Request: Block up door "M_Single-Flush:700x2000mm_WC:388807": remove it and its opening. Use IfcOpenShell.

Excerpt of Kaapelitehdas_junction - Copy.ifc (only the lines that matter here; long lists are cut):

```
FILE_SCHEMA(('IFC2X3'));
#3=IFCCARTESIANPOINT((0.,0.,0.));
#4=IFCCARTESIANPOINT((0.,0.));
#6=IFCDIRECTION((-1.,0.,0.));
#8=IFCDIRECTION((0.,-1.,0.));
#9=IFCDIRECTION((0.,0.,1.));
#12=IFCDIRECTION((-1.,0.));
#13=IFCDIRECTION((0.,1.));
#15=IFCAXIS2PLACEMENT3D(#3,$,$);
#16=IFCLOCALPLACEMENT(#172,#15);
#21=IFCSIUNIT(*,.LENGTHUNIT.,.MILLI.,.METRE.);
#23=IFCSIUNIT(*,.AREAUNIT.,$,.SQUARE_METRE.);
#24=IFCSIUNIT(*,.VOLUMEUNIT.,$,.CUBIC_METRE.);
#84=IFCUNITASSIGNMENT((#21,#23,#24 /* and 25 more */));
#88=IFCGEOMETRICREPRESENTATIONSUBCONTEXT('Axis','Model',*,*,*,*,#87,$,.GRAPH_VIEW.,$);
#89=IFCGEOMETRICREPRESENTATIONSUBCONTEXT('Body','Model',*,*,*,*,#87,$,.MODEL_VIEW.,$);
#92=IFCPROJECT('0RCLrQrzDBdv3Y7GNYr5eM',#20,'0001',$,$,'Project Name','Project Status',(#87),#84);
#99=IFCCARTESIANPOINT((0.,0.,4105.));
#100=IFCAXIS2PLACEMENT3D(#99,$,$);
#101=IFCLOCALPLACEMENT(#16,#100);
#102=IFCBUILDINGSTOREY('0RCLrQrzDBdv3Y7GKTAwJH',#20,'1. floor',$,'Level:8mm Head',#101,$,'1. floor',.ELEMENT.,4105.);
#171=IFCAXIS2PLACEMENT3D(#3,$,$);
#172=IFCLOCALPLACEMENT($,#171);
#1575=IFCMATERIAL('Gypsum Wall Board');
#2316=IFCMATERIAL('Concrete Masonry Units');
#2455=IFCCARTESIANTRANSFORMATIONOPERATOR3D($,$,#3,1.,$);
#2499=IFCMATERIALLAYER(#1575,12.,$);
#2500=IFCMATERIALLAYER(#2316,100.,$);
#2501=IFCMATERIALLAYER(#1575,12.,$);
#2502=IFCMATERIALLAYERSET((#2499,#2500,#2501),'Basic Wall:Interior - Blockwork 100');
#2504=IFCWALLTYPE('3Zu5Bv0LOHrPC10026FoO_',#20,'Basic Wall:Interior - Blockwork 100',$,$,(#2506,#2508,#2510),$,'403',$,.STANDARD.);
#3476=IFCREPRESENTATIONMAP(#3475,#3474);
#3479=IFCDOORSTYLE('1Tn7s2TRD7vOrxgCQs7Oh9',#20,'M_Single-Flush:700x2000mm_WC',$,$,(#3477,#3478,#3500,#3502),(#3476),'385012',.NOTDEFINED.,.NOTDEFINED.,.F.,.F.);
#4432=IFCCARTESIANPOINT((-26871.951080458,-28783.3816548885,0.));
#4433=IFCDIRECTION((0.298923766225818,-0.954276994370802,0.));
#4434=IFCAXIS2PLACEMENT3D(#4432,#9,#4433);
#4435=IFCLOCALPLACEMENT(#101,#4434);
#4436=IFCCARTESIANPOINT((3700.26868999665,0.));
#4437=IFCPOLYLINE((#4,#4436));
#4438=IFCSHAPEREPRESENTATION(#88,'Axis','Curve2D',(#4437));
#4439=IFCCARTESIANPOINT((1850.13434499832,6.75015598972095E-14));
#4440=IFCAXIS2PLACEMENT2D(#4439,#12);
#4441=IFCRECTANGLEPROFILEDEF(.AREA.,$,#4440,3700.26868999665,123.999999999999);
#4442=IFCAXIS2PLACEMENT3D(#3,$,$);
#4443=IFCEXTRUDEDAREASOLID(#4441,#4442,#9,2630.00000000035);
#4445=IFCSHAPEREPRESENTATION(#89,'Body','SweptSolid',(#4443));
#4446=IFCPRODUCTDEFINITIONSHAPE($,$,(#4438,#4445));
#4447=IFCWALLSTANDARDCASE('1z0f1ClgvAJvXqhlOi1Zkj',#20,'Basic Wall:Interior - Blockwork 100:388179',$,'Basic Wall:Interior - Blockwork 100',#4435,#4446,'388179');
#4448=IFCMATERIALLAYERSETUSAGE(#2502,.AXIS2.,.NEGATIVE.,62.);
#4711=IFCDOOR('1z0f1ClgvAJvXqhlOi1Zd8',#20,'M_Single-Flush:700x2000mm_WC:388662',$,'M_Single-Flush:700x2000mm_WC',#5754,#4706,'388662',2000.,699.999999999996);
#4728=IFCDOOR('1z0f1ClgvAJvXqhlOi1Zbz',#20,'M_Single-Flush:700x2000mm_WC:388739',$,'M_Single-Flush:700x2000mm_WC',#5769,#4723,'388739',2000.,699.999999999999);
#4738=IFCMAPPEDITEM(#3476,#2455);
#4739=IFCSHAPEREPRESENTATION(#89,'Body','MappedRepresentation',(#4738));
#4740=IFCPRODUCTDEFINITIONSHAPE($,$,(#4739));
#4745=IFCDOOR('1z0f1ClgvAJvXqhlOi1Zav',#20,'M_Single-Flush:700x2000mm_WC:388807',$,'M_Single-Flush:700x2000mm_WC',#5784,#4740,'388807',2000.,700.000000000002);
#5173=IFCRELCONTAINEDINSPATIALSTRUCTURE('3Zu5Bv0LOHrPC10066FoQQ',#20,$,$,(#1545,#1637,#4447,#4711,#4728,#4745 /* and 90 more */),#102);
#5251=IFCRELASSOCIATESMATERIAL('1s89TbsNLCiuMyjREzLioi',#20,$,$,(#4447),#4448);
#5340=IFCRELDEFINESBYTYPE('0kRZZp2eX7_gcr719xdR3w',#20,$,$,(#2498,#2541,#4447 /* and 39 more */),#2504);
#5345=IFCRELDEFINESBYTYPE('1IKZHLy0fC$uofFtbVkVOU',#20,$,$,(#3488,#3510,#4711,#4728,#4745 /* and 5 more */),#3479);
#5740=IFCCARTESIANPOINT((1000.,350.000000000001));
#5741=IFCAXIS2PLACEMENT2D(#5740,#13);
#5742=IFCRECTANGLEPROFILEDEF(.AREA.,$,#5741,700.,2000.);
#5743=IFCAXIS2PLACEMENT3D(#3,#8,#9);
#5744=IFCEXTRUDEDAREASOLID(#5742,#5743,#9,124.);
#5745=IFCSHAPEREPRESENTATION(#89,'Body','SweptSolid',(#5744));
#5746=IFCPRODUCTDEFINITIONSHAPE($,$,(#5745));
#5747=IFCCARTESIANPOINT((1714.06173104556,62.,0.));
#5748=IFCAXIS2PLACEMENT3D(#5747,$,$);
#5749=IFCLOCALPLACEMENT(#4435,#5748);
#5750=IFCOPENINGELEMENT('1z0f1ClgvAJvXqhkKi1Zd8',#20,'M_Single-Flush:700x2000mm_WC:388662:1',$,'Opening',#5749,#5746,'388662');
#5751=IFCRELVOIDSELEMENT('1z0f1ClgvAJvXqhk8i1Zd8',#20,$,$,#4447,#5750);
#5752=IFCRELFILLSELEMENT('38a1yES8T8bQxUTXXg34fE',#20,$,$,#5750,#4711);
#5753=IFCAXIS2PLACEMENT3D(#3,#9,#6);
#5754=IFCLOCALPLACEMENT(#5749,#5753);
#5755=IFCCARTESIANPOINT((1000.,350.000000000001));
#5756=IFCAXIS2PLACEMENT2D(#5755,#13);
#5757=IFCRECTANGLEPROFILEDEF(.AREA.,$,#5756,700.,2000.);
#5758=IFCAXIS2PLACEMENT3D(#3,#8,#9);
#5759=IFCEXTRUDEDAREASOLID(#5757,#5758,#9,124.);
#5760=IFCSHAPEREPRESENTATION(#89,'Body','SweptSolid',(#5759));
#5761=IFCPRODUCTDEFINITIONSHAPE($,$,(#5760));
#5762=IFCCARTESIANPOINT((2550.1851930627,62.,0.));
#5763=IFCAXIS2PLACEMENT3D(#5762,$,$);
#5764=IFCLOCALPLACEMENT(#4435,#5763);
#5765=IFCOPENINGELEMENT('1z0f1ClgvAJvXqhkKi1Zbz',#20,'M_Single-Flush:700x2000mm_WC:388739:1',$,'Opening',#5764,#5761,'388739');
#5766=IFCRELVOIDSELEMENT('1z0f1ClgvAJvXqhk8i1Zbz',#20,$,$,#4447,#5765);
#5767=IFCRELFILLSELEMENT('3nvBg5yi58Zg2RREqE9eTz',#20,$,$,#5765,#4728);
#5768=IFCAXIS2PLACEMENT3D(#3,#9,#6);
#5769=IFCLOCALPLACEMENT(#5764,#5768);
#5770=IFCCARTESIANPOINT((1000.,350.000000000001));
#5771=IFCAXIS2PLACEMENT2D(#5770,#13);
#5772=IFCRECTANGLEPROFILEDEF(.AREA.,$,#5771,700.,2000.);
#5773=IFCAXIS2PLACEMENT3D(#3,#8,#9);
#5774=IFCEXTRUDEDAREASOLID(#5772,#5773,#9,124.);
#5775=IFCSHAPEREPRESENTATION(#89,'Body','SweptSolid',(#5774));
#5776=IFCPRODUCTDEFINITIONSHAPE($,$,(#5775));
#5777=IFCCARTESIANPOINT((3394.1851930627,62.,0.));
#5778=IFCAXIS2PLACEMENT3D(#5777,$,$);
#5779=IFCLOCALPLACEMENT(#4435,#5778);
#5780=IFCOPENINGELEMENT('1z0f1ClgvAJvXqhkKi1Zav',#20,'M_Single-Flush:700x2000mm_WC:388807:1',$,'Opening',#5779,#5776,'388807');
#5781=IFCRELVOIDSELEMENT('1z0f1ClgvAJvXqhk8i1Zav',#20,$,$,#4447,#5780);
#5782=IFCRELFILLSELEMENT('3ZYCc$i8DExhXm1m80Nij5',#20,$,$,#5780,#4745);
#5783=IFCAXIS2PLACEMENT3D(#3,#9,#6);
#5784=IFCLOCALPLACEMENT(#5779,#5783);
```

```python
import ifcopenshell
import ifcopenshell.api.feature
import ifcopenshell.api.root
import ifcopenshell.geom
import ifcopenshell.util.shape

model = ifcopenshell.open("Kaapelitehdas_junction - Copy.ifc")
settings = ifcopenshell.geom.settings()


def volume(element):
    """Net volume in cubic metres, openings subtracted."""
    shape = ifcopenshell.geom.create_shape(settings, element)
    return ifcopenshell.util.shape.get_volume(shape.geometry)


door = model.by_guid("1z0f1ClgvAJvXqhlOi1Zav")
opening = door.FillsVoids[0].RelatingOpeningElement
wall = opening.VoidsElements[0].RelatingBuildingElement
before = volume(wall)

ifcopenshell.api.root.remove_product(model, product=door)
ifcopenshell.api.feature.remove_feature(model, feature=opening)

after = volume(wall)

print(f"wall volume {before:.3f} -> {after:.3f} m3")

model.write("Kaapelitehdas_junction - Copy-out.ifc")
```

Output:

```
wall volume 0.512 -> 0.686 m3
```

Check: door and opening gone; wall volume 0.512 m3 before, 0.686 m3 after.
